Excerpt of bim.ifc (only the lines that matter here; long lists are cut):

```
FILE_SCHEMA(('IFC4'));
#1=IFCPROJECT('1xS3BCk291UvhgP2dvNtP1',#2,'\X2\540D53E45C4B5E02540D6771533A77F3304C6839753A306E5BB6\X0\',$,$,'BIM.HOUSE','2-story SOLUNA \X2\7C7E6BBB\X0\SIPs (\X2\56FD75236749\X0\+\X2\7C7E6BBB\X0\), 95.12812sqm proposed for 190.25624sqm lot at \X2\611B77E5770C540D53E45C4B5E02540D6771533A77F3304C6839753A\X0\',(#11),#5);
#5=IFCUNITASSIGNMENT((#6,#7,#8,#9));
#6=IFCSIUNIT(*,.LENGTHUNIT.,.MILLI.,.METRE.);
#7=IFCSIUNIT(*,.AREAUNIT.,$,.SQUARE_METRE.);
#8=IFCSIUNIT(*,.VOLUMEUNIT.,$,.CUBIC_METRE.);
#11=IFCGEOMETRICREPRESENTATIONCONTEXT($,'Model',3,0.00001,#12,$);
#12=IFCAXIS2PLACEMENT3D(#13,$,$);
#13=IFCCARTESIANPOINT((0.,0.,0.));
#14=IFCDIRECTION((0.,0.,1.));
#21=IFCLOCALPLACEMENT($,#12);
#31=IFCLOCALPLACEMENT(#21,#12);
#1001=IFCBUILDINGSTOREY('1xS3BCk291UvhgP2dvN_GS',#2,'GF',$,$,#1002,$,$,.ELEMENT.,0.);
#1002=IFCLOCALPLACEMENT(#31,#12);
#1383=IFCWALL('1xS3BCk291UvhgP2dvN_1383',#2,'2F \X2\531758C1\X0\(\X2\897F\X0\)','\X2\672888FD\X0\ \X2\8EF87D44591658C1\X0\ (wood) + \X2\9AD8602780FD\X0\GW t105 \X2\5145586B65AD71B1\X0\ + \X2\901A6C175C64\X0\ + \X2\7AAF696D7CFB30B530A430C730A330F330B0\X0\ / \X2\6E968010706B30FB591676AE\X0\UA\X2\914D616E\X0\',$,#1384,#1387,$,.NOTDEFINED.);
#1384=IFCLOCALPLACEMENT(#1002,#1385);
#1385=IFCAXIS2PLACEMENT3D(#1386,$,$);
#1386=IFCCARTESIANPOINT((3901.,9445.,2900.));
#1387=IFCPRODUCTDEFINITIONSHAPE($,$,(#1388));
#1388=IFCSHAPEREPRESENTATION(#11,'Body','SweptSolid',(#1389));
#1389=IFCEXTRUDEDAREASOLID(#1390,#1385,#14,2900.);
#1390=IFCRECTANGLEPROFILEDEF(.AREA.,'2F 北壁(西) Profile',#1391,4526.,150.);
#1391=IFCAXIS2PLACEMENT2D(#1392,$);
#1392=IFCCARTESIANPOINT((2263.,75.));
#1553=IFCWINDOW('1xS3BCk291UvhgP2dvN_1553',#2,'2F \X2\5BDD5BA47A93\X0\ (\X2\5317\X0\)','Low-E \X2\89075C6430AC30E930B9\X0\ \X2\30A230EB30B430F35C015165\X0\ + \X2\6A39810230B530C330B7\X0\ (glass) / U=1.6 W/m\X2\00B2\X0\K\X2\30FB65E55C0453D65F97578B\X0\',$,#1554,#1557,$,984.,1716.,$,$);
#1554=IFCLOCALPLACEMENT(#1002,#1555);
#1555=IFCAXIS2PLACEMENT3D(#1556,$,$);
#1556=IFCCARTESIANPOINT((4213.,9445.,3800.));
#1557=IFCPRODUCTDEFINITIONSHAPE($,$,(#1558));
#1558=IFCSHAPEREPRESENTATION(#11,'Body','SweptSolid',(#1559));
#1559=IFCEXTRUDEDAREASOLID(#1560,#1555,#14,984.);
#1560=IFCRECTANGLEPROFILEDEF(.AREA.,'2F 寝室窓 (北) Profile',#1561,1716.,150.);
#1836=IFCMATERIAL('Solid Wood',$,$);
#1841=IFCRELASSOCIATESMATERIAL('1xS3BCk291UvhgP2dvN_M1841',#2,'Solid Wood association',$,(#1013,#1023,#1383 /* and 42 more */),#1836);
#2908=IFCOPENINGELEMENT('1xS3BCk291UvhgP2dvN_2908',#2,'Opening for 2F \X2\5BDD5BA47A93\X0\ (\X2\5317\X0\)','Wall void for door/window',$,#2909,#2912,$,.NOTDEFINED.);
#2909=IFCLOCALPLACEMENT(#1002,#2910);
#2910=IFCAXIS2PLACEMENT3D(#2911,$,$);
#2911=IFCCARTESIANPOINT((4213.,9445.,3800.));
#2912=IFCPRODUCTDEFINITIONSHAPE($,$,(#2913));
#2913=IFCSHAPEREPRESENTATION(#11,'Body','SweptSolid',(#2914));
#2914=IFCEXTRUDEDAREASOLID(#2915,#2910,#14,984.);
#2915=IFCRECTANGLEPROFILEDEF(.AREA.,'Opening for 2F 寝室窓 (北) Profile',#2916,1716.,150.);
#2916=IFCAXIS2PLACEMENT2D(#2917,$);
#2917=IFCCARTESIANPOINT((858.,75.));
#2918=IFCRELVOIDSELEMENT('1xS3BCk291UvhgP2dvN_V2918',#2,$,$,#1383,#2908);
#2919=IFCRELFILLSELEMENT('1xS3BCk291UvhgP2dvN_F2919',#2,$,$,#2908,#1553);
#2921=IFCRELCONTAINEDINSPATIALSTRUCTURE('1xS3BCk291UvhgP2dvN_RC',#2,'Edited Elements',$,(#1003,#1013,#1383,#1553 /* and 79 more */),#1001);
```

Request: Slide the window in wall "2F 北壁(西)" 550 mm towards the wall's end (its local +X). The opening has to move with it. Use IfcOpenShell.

```python
import ifcopenshell
import ifcopenshell.api.geometry
import ifcopenshell.util.placement
import ifcopenshell.util.unit

model = ifcopenshell.open("bim.ifc")
unit_scale = ifcopenshell.util.unit.calculate_unit_scale(model)

window = model.by_id(1553)
opening = window.FillsVoids[0].RelatingOpeningElement
wall = opening.VoidsElements[0].RelatingBuildingElement

wall_matrix = ifcopenshell.util.placement.get_local_placement(wall.ObjectPlacement)
shift = wall_matrix[:3, 0] * 0.55 / unit_scale
before = ifcopenshell.util.placement.get_local_placement(window.ObjectPlacement)[:3, 3].copy()

# The window is not placed relative to its opening, so move both.
for product in (opening, window):
    matrix = ifcopenshell.util.placement.get_local_placement(product.ObjectPlacement)
    matrix[:3, 3] += shift
    ifcopenshell.api.geometry.edit_object_placement(model, product=product, matrix=matrix, is_si=False)

after = ifcopenshell.util.placement.get_local_placement(window.ObjectPlacement)[:3, 3]
print("window moved by", (after - before).round(3) + 0.0)

model.write("bim-out.ifc")
```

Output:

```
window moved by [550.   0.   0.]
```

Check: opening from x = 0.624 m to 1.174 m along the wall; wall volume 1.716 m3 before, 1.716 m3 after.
